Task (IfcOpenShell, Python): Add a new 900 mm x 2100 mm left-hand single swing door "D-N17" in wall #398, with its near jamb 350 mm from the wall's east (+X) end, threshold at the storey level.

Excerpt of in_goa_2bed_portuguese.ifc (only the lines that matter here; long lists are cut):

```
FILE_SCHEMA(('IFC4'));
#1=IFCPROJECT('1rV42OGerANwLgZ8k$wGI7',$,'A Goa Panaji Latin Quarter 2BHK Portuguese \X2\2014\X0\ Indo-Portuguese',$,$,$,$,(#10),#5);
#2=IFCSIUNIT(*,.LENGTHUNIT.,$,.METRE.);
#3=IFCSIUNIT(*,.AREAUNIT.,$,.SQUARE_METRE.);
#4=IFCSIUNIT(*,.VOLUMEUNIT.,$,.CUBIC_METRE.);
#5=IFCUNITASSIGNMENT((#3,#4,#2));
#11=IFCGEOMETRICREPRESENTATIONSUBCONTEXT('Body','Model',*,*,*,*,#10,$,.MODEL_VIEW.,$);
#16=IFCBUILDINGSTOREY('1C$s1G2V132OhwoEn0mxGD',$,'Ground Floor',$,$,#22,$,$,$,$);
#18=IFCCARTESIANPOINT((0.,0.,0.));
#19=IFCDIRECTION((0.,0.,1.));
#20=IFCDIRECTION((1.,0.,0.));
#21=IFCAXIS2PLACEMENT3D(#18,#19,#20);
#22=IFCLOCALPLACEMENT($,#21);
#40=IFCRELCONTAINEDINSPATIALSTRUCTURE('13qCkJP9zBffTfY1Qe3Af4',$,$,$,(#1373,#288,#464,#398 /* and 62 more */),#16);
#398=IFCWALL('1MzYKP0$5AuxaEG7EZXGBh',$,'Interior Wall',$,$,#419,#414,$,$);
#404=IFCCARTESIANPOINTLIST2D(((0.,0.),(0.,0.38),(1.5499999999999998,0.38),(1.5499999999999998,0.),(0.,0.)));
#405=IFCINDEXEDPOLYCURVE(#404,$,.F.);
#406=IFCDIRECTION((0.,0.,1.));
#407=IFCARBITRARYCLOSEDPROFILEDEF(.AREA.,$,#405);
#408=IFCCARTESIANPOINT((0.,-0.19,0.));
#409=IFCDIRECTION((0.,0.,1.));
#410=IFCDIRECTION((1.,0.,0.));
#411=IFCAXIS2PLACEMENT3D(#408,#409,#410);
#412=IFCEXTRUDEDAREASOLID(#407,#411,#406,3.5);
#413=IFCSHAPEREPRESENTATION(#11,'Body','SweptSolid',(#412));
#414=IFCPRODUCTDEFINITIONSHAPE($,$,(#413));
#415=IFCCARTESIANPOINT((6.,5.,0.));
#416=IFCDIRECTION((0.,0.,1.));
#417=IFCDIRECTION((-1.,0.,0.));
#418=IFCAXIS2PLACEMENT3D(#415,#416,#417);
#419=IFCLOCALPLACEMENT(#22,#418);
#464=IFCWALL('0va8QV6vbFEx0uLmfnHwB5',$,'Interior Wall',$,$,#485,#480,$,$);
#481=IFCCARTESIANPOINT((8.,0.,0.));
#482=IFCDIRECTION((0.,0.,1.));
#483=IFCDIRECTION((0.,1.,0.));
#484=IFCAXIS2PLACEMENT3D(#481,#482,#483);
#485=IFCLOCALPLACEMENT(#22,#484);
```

```python
import numpy as np
import ifcopenshell
import ifcopenshell.api.feature
import ifcopenshell.api.geometry
import ifcopenshell.api.root
import ifcopenshell.api.spatial
import ifcopenshell.geom
import ifcopenshell.util.element
import ifcopenshell.util.placement
import ifcopenshell.util.representation
import ifcopenshell.util.shape
import ifcopenshell.util.unit

model = ifcopenshell.open("in_goa_2bed_portuguese.ifc")
unit_scale = ifcopenshell.util.unit.calculate_unit_scale(model)
settings = ifcopenshell.geom.settings()


def volume(element):
    """Net volume in cubic metres, openings subtracted."""
    shape = ifcopenshell.geom.create_shape(settings, element)
    return ifcopenshell.util.shape.get_volume(shape.geometry)


wall = model.by_guid("1MzYKP0$5AuxaEG7EZXGBh")
storey = ifcopenshell.util.element.get_container(wall, ifc_class="IfcBuildingStorey")
context = ifcopenshell.util.representation.get_context(model, "Model", "Body", "MODEL_VIEW")
before = volume(wall)

width, height, from_end, sill = 0.9, 2.1, 0.35, 0.0  # metres

# The wall runs along its own X axis, and the end named is its -X end.
wall_shape = ifcopenshell.geom.create_shape(settings, wall)
x, y, z = ifcopenshell.util.shape.get_vertices(wall_shape.geometry).T
start = x.min() + from_end
face, thickness = float(y.min()), float(y.max() - y.min())
wall_matrix = ifcopenshell.util.placement.get_local_placement(wall.ObjectPlacement)
level = ifcopenshell.util.placement.get_local_placement(storey.ObjectPlacement)[2, 3]


def in_wall(x, y):
    """Placement at x, y metres in the wall's axes, at sill height."""
    matrix = wall_matrix.copy()
    matrix[:, 3] = wall_matrix @ np.array([x / unit_scale, y / unit_scale, 0.0, 1.0])
    matrix[2, 3] = level + sill / unit_scale
    return matrix


# Opening: a box that overshoots both wall faces by 50 mm.
opening = ifcopenshell.api.root.create_entity(model, ifc_class="IfcOpeningElement", predefined_type="OPENING")
box = ifcopenshell.api.geometry.add_wall_representation(
    model, context=context, length=width, height=height, thickness=thickness + 0.1
)
ifcopenshell.api.geometry.assign_representation(model, product=opening, representation=box)
ifcopenshell.api.geometry.edit_object_placement(model, product=opening, matrix=in_wall(start, face - 0.05), is_si=False)
ifcopenshell.api.feature.add_feature(model, feature=opening, element=wall)

door = ifcopenshell.api.root.create_entity(model, ifc_class="IfcDoor", name="D-N17", predefined_type="DOOR")
door.OverallWidth, door.OverallHeight = width / unit_scale, height / unit_scale
door.OperationType = "SINGLE_SWING_LEFT"
body = ifcopenshell.api.geometry.add_door_representation(
    model,
    context=context,
    overall_width=door.OverallWidth,
    overall_height=door.OverallHeight,
    operation_type="SINGLE_SWING_LEFT",
    lining_properties={"LiningDepth": thickness / unit_scale, "ThresholdDepth": thickness / unit_scale},
)
ifcopenshell.api.geometry.assign_representation(model, product=door, representation=body)
ifcopenshell.api.spatial.assign_container(model, products=[door], relating_structure=storey)
ifcopenshell.api.feature.add_filling(model, opening=opening, element=door)

# The lining spans the wall, so the door starts at the wall face.
ifcopenshell.api.geometry.edit_object_placement(model, product=door, matrix=in_wall(start, face), is_si=False)

after = volume(wall)

print(f"wall volume {before:.3f} -> {after:.3f} m3")

model.write("in_goa_2bed_portuguese_edited.ifc")
```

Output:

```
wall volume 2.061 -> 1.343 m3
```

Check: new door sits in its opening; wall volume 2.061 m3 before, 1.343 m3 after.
